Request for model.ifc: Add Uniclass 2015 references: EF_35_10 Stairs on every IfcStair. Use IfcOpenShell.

First a look at what the model holds.

```python
import ifcopenshell

model = ifcopenshell.open("model.ifc")
print(model.schema)
print("classifications:", [c.Name for c in model.by_type("IfcClassification")])
for ifc_class in ("IfcDoor", "IfcRoof", "IfcStair", "IfcWall", "IfcWindow"):
    print(ifc_class, len(model.by_type(ifc_class)))
```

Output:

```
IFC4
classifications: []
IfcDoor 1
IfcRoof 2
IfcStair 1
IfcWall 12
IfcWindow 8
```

```python
import ifcopenshell
import ifcopenshell.api.classification

model = ifcopenshell.open("model.ifc")

system = ifcopenshell.api.classification.add_classification(model, classification="Uniclass 2015")

codes = {
    "IfcStair": ("EF_35_10", "Stairs"),
}
for ifc_class, (code, name) in codes.items():
    products = model.by_type(ifc_class)
    ifcopenshell.api.classification.add_reference(
        model, products=products, classification=system, identification=code, name=name
    )
    print(code, len(products))

model.write("model_rev.ifc")
```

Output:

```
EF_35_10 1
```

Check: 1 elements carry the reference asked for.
